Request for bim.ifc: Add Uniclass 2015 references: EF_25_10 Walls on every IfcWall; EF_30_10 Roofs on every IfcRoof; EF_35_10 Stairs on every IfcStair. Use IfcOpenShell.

First a look at what the model holds.

```python
import ifcopenshell

model = ifcopenshell.open("bim.ifc")
print(model.schema)
print("classifications:", [c.Name for c in model.by_type("IfcClassification")])
for ifc_class in ("IfcDoor", "IfcRoof", "IfcStair", "IfcWall", "IfcWindow"):
    print(ifc_class, len(model.by_type(ifc_class)))
```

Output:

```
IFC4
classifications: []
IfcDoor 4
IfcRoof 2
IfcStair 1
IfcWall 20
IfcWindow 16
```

```python
import ifcopenshell
import ifcopenshell.api.classification

model = ifcopenshell.open("bim.ifc")

system = ifcopenshell.api.classification.add_classification(model, classification="Uniclass 2015")

codes = {
    "IfcWall": ("EF_25_10", "Walls"),
    "IfcRoof": ("EF_30_10", "Roofs"),
    "IfcStair": ("EF_35_10", "Stairs"),
}
for ifc_class, (code, name) in codes.items():
    products = model.by_type(ifc_class)
    ifcopenshell.api.classification.add_reference(
        model, products=products, classification=system, identification=code, name=name
    )
    print(code, len(products))

model.write("bim_rev.ifc")
```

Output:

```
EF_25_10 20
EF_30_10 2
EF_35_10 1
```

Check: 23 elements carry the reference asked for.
